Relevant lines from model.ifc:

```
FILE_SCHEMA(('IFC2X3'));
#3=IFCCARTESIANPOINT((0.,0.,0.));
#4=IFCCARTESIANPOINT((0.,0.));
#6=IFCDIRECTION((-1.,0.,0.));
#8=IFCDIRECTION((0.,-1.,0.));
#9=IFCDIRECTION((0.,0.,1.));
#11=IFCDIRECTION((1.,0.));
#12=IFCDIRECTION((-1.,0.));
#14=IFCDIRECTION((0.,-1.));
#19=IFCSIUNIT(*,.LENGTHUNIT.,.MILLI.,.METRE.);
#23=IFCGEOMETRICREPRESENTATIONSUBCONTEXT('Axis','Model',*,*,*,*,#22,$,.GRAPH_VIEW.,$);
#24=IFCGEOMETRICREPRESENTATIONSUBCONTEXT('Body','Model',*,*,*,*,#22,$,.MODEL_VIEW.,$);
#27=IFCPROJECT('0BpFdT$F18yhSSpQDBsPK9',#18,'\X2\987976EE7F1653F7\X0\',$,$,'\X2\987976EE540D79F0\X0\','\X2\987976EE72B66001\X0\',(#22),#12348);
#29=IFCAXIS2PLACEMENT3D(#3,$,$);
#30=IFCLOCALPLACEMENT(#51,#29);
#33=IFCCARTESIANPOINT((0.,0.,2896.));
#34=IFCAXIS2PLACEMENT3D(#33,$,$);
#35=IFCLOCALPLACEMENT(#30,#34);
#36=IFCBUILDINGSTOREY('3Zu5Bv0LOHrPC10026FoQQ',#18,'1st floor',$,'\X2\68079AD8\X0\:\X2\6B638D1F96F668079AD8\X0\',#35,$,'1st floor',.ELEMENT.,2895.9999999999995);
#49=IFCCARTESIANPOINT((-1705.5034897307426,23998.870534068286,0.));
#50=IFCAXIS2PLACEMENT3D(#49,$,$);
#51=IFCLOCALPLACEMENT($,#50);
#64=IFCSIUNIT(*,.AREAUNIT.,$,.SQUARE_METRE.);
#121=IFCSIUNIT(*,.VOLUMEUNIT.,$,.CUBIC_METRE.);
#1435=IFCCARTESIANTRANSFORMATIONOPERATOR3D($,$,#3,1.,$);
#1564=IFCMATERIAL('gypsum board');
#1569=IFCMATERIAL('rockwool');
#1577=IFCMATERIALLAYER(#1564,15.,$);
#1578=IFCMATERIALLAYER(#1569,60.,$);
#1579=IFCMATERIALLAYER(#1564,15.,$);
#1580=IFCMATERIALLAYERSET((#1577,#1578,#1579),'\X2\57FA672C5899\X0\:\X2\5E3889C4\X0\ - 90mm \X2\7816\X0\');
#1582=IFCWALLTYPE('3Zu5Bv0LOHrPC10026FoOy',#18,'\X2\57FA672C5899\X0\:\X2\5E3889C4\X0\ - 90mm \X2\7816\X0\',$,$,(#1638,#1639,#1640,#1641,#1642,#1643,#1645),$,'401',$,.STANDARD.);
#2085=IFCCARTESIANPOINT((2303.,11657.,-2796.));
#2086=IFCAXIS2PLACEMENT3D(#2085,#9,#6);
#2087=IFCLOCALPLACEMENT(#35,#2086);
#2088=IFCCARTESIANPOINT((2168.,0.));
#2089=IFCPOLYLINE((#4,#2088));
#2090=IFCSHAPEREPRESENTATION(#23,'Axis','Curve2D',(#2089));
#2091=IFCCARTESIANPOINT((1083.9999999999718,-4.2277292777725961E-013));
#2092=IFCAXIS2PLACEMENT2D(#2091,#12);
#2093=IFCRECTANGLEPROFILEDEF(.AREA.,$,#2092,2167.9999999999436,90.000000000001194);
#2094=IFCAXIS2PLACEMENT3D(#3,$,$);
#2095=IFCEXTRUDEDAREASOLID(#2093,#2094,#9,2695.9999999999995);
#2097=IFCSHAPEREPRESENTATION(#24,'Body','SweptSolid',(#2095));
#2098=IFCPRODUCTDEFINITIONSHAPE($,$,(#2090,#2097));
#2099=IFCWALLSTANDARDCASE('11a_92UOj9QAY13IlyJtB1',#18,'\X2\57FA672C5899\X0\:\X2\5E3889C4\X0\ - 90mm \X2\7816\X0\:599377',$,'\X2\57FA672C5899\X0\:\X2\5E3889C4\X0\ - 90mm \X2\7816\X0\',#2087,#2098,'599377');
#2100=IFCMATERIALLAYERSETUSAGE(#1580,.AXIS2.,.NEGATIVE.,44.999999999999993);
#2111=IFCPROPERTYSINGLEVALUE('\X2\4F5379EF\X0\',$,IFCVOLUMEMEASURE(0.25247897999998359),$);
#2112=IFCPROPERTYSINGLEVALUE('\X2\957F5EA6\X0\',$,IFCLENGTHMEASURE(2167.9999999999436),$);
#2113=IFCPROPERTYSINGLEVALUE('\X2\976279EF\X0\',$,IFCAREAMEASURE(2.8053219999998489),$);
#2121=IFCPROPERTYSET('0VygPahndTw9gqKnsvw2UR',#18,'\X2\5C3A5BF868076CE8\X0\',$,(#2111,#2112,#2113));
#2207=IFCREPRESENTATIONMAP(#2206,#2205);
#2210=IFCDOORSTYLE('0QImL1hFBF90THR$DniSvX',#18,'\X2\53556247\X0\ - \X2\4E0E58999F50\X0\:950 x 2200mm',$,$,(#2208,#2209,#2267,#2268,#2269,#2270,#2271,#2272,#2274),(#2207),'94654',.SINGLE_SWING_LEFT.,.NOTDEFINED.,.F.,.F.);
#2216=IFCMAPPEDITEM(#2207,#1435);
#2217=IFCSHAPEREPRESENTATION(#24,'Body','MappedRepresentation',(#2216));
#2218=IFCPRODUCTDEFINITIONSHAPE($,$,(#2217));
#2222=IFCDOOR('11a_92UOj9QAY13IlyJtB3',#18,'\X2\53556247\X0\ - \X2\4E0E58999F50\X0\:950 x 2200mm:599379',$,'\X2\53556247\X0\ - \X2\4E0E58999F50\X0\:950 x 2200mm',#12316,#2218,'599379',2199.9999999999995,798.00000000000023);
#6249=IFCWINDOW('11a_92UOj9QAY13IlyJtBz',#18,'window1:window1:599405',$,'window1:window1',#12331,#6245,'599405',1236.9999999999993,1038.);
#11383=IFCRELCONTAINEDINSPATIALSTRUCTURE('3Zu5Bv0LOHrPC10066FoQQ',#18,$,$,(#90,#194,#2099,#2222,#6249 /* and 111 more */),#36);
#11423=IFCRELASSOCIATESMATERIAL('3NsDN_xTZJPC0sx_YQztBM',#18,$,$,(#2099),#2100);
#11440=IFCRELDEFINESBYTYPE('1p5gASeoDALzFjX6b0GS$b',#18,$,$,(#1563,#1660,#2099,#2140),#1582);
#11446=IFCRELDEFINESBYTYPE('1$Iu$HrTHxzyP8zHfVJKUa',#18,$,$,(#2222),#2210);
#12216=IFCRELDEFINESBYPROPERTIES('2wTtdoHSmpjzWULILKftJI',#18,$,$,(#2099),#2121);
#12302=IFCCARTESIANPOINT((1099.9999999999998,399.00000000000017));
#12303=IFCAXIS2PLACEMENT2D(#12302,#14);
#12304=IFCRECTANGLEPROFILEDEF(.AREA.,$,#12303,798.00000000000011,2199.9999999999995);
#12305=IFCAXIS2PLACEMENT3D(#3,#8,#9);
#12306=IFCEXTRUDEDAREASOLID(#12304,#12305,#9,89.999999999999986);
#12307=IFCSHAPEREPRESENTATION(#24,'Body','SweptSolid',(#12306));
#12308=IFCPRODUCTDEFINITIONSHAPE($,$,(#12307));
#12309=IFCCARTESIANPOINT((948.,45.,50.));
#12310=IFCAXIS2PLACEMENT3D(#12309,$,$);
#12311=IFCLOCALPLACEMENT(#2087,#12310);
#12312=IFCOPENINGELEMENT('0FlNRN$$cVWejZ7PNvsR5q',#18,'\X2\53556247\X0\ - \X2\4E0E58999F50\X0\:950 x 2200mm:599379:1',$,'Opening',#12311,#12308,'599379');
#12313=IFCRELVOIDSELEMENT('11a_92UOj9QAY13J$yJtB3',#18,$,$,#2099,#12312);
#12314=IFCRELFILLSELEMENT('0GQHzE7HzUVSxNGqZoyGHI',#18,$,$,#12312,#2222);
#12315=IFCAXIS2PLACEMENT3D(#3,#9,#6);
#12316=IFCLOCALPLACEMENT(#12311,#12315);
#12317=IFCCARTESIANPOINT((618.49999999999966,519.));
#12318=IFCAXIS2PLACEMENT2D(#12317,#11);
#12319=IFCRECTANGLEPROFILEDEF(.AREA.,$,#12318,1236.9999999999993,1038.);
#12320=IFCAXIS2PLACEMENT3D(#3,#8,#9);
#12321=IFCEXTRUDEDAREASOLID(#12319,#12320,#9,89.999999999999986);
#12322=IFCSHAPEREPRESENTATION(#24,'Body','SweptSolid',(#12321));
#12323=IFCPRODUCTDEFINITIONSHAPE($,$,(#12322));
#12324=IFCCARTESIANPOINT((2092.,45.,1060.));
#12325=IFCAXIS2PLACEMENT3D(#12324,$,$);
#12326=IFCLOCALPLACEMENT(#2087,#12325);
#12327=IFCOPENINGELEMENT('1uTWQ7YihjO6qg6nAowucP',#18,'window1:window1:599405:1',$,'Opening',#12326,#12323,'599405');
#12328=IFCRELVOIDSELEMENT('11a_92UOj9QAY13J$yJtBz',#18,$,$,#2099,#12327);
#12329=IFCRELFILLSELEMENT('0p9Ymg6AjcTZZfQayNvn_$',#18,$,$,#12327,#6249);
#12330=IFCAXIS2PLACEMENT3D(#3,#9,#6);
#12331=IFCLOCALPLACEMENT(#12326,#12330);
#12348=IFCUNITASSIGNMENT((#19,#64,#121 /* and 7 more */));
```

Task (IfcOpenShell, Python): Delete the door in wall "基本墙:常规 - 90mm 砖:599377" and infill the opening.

```python
import ifcopenshell
import ifcopenshell.api.feature
import ifcopenshell.api.pset
import ifcopenshell.api.root
import ifcopenshell.geom
import ifcopenshell.util.element
import ifcopenshell.util.shape
import ifcopenshell.util.unit

model = ifcopenshell.open("model.ifc")
area_scale = ifcopenshell.util.unit.calculate_unit_scale(model, "AREAUNIT")
volume_scale = ifcopenshell.util.unit.calculate_unit_scale(model, "VOLUMEUNIT")
settings = ifcopenshell.geom.settings()


def volume(element):
    """Net volume in cubic metres, openings subtracted."""
    shape = ifcopenshell.geom.create_shape(settings, element)
    return ifcopenshell.util.shape.get_volume(shape.geometry)


door = model.by_id(2222)
opening = door.FillsVoids[0].RelatingOpeningElement
wall = opening.VoidsElements[0].RelatingBuildingElement
before = volume(wall)

ifcopenshell.api.root.remove_product(model, product=door)
ifcopenshell.api.feature.remove_feature(model, feature=opening)

after = volume(wall)
thickness = 0.09  # wall thickness in metres

# Update the wall's stored quantities.
pset = model.by_id(ifcopenshell.util.element.get_pset(wall, "尺寸标注", should_inherit=False)["id"])
ifcopenshell.api.pset.edit_pset(model, pset=pset, properties={
    "体积": model.create_entity("IfcVolumeMeasure", after / volume_scale),
    "面积": model.create_entity("IfcAreaMeasure", after / thickness / area_scale),
})

print(f"wall volume {before:.3f} -> {after:.3f} m3")

model.write("model_edited.ifc")
```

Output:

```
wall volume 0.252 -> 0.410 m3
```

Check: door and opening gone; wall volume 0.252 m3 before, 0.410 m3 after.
